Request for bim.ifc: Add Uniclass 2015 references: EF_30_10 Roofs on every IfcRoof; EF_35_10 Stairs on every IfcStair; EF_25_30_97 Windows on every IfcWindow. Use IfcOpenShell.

First a look at what the model holds.

```python
import ifcopenshell

model = ifcopenshell.open("bim.ifc")
print(model.schema)
print("classifications:", [c.Name for c in model.by_type("IfcClassification")])
for ifc_class in ("IfcDoor", "IfcRoof", "IfcStair", "IfcWall", "IfcWindow"):
    print(ifc_class, len(model.by_type(ifc_class)))
```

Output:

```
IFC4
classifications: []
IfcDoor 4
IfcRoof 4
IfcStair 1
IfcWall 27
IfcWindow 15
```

```python
import ifcopenshell
import ifcopenshell.api.classification

model = ifcopenshell.open("bim.ifc")

system = ifcopenshell.api.classification.add_classification(model, classification="Uniclass 2015")

codes = {
    "IfcRoof": ("EF_30_10", "Roofs"),
    "IfcStair": ("EF_35_10", "Stairs"),
    "IfcWindow": ("EF_25_30_97", "Windows"),
}
for ifc_class, (code, name) in codes.items():
    products = model.by_type(ifc_class)
    ifcopenshell.api.classification.add_reference(
        model, products=products, classification=system, identification=code, name=name
    )
    print(code, len(products))

model.write("bim-out.ifc")
```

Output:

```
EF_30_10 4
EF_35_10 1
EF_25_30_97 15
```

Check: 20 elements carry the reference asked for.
